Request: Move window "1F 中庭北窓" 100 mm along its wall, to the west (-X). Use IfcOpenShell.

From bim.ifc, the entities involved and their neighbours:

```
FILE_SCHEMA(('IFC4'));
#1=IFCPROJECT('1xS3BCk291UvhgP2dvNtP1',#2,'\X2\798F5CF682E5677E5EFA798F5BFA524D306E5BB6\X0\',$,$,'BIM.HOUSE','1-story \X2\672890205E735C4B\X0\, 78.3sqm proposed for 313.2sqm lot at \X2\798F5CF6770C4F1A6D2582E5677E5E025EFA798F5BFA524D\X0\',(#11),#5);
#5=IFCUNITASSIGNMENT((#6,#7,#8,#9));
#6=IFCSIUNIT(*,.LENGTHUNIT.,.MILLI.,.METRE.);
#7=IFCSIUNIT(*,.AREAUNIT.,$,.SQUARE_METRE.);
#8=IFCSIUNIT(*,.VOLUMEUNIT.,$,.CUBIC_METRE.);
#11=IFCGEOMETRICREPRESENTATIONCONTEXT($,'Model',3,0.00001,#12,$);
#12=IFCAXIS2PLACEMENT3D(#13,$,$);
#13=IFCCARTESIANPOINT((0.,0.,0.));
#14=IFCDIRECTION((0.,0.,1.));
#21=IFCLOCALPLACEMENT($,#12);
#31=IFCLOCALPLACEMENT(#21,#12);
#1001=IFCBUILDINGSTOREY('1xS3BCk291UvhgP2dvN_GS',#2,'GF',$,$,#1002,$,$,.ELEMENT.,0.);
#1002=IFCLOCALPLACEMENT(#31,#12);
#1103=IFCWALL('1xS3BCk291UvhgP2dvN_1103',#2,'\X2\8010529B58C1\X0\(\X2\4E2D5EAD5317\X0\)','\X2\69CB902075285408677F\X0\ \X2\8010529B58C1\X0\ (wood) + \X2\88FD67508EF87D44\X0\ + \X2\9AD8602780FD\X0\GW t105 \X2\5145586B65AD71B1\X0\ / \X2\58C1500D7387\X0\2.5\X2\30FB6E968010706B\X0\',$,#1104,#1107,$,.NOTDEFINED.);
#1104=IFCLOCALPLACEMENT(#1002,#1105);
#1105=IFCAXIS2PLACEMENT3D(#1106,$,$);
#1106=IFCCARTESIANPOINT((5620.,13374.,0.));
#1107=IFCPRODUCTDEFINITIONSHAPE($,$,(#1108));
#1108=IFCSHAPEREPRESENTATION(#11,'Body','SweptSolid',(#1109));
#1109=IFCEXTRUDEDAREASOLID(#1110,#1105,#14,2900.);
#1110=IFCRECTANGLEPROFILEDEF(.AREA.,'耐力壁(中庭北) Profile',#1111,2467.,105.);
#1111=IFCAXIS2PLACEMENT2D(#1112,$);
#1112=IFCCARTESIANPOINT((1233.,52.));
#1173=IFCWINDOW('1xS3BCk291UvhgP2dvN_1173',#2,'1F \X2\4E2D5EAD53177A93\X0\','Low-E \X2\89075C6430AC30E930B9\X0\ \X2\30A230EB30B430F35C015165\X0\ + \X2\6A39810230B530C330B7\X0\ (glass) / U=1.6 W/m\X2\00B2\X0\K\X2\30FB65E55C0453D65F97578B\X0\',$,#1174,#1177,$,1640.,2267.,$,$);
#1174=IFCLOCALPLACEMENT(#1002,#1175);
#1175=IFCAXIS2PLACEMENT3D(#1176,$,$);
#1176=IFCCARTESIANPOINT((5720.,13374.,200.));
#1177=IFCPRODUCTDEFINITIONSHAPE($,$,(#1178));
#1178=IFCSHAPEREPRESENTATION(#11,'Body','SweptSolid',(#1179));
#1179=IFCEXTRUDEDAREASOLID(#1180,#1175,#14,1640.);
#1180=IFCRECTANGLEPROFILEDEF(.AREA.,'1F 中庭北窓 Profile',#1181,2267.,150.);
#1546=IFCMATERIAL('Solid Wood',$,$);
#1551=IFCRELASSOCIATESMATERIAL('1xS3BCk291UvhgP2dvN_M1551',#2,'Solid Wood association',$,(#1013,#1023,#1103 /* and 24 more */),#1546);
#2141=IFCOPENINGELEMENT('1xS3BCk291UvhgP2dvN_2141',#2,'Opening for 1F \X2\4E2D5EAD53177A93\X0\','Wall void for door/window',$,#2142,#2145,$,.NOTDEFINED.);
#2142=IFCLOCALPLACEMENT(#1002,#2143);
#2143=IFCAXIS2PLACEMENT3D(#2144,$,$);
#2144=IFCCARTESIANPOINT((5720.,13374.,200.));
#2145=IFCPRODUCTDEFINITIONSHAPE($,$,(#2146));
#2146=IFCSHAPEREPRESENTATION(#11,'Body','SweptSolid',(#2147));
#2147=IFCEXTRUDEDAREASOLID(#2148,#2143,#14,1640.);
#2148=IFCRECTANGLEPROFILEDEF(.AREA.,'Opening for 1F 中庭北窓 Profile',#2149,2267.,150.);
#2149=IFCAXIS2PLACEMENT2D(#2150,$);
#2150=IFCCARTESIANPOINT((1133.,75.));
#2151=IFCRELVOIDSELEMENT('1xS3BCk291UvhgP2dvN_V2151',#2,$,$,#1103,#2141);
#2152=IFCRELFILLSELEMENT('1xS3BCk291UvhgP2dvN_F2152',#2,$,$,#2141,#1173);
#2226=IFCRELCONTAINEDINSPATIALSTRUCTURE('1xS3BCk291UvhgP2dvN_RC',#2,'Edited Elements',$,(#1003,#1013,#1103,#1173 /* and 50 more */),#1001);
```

```python
import ifcopenshell
import ifcopenshell.api.geometry
import ifcopenshell.util.placement

model = ifcopenshell.open("bim.ifc")

window = model.by_id(1173)
opening = window.FillsVoids[0].RelatingOpeningElement
wall = opening.VoidsElements[0].RelatingBuildingElement

wall_matrix = ifcopenshell.util.placement.get_local_placement(wall.ObjectPlacement)
shift = wall_matrix[:3, 0] * -100.0
before = ifcopenshell.util.placement.get_local_placement(window.ObjectPlacement)[:3, 3].copy()

# The window is not placed relative to its opening, so move both.
for product in (opening, window):
    matrix = ifcopenshell.util.placement.get_local_placement(product.ObjectPlacement)
    matrix[:3, 3] += shift
    ifcopenshell.api.geometry.edit_object_placement(model, product=product, matrix=matrix, is_si=False)

after = ifcopenshell.util.placement.get_local_placement(window.ObjectPlacement)[:3, 3]
print("window moved by", (after - before).round(3) + 0.0)

model.write("bim_v2.ifc")
```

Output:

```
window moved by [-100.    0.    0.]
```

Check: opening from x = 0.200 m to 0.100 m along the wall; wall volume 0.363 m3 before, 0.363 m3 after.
